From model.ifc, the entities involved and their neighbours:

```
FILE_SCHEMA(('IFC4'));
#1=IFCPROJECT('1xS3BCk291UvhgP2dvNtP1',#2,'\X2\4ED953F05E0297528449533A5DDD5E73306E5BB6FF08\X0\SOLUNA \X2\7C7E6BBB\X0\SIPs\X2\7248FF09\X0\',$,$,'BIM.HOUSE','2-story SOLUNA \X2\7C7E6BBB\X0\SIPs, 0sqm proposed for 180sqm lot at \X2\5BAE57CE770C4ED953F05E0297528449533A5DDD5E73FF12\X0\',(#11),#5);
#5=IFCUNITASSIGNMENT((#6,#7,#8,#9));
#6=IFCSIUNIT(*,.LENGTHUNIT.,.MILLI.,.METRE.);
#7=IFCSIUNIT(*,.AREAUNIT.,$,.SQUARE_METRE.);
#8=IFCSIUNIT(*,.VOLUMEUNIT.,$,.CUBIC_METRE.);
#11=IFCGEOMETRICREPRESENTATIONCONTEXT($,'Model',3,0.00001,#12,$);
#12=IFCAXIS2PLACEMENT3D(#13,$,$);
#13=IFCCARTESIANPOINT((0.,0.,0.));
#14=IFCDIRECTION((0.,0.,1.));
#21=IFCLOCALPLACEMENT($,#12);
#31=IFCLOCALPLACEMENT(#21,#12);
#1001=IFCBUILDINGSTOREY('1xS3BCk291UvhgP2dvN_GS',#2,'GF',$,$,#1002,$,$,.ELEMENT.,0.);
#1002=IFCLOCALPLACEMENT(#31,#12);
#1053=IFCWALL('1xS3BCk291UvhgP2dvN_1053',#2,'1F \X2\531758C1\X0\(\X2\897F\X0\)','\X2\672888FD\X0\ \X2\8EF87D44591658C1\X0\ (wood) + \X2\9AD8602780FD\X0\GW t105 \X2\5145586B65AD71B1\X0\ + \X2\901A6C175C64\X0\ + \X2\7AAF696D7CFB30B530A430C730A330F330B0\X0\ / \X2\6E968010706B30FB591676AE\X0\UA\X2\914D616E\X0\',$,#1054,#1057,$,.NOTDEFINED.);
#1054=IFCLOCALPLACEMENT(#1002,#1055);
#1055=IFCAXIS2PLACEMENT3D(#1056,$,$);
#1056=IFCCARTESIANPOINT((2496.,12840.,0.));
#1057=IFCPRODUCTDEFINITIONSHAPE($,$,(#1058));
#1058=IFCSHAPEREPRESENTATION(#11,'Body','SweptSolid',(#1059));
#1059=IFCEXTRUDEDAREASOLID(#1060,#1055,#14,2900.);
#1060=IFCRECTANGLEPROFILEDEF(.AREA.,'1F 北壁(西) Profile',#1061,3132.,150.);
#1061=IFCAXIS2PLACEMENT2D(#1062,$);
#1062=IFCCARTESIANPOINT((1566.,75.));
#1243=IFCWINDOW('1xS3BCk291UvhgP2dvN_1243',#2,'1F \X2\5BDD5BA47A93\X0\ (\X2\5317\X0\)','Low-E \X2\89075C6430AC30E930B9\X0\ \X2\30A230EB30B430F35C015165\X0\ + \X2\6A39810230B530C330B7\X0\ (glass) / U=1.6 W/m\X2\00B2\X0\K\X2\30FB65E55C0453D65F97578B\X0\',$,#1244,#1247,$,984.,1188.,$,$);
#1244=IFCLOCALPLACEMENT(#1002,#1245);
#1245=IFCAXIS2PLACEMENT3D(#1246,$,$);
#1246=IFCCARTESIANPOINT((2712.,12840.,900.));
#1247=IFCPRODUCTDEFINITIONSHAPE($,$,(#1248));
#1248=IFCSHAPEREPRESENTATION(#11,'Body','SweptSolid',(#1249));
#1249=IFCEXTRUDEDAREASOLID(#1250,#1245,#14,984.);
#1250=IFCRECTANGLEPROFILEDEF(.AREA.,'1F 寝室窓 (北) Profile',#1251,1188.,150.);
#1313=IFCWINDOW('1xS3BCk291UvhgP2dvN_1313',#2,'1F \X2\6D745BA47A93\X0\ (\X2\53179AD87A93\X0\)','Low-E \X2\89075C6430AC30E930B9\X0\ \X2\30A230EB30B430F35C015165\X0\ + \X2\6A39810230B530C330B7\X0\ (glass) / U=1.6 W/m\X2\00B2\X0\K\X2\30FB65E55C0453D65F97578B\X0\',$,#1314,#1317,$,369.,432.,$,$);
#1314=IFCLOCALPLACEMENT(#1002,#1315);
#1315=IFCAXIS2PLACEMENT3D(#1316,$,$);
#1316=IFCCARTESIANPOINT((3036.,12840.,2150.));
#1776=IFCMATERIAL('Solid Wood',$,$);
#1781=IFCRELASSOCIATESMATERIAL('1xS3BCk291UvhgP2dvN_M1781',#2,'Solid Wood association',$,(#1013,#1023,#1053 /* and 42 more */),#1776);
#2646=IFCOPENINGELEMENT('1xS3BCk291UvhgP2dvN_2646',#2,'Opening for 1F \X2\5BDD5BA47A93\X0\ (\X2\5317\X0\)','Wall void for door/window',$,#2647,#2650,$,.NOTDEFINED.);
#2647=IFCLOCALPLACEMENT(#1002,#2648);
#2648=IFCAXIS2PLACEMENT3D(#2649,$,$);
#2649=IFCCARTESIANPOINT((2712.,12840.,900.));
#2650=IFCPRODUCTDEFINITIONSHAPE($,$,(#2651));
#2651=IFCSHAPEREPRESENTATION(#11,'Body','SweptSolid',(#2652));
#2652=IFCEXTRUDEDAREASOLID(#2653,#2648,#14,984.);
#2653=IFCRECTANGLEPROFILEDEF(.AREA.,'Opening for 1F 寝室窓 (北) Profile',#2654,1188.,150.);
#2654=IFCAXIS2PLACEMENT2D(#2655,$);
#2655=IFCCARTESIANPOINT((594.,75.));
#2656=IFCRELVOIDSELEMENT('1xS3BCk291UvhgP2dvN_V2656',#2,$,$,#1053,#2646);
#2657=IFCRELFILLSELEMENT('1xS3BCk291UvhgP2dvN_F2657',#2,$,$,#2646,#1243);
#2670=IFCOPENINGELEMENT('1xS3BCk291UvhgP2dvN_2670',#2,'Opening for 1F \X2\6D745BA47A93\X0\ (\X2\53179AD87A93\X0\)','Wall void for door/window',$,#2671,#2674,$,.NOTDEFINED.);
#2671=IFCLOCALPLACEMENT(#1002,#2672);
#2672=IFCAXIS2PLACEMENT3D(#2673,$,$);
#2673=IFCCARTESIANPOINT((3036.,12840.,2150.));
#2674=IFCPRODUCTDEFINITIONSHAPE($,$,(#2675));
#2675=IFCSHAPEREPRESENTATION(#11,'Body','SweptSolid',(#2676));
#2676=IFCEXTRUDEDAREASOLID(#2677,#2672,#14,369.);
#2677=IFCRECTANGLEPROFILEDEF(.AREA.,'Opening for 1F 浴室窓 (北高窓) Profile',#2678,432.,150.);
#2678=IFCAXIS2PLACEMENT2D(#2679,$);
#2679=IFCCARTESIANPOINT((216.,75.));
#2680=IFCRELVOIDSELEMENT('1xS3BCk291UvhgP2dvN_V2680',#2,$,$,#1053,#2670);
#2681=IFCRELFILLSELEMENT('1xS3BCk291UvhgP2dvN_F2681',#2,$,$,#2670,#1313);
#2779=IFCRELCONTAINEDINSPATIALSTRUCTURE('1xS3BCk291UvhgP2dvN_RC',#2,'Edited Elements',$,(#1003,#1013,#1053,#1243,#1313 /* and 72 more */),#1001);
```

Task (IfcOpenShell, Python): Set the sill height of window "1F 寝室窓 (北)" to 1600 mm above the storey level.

```python
import numpy as np
import ifcopenshell
import ifcopenshell.api.geometry
import ifcopenshell.geom
import ifcopenshell.util.element
import ifcopenshell.util.placement
import ifcopenshell.util.shape
import ifcopenshell.util.unit

model = ifcopenshell.open("model.ifc")
unit_scale = ifcopenshell.util.unit.calculate_unit_scale(model)

window = model.by_guid("1xS3BCk291UvhgP2dvN_1243")
opening = window.FillsVoids[0].RelatingOpeningElement
storey = ifcopenshell.util.element.get_container(window, ifc_class="IfcBuildingStorey")
level = ifcopenshell.util.placement.get_local_placement(storey.ObjectPlacement)[2, 3]

# The opening's origin need not be at the sill, so measure its lowest point.
shape = ifcopenshell.geom.create_shape(ifcopenshell.geom.settings(), opening)
bottom = ifcopenshell.util.shape.get_shape_bottom_elevation(shape, shape.geometry) / unit_scale
dz = level + 1.6 / unit_scale - bottom

shift = np.array([0.0, 0.0, dz])
# The window is not placed relative to its opening, so move both.
for product in (opening, window):
    matrix = ifcopenshell.util.placement.get_local_placement(product.ObjectPlacement)
    matrix[:3, 3] += shift
    ifcopenshell.api.geometry.edit_object_placement(model, product=product, matrix=matrix, is_si=False)

print(f"moved by {dz * unit_scale:+.3f} m")

model.write("model_edited.ifc")
```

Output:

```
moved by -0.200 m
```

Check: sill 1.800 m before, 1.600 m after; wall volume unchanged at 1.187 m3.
